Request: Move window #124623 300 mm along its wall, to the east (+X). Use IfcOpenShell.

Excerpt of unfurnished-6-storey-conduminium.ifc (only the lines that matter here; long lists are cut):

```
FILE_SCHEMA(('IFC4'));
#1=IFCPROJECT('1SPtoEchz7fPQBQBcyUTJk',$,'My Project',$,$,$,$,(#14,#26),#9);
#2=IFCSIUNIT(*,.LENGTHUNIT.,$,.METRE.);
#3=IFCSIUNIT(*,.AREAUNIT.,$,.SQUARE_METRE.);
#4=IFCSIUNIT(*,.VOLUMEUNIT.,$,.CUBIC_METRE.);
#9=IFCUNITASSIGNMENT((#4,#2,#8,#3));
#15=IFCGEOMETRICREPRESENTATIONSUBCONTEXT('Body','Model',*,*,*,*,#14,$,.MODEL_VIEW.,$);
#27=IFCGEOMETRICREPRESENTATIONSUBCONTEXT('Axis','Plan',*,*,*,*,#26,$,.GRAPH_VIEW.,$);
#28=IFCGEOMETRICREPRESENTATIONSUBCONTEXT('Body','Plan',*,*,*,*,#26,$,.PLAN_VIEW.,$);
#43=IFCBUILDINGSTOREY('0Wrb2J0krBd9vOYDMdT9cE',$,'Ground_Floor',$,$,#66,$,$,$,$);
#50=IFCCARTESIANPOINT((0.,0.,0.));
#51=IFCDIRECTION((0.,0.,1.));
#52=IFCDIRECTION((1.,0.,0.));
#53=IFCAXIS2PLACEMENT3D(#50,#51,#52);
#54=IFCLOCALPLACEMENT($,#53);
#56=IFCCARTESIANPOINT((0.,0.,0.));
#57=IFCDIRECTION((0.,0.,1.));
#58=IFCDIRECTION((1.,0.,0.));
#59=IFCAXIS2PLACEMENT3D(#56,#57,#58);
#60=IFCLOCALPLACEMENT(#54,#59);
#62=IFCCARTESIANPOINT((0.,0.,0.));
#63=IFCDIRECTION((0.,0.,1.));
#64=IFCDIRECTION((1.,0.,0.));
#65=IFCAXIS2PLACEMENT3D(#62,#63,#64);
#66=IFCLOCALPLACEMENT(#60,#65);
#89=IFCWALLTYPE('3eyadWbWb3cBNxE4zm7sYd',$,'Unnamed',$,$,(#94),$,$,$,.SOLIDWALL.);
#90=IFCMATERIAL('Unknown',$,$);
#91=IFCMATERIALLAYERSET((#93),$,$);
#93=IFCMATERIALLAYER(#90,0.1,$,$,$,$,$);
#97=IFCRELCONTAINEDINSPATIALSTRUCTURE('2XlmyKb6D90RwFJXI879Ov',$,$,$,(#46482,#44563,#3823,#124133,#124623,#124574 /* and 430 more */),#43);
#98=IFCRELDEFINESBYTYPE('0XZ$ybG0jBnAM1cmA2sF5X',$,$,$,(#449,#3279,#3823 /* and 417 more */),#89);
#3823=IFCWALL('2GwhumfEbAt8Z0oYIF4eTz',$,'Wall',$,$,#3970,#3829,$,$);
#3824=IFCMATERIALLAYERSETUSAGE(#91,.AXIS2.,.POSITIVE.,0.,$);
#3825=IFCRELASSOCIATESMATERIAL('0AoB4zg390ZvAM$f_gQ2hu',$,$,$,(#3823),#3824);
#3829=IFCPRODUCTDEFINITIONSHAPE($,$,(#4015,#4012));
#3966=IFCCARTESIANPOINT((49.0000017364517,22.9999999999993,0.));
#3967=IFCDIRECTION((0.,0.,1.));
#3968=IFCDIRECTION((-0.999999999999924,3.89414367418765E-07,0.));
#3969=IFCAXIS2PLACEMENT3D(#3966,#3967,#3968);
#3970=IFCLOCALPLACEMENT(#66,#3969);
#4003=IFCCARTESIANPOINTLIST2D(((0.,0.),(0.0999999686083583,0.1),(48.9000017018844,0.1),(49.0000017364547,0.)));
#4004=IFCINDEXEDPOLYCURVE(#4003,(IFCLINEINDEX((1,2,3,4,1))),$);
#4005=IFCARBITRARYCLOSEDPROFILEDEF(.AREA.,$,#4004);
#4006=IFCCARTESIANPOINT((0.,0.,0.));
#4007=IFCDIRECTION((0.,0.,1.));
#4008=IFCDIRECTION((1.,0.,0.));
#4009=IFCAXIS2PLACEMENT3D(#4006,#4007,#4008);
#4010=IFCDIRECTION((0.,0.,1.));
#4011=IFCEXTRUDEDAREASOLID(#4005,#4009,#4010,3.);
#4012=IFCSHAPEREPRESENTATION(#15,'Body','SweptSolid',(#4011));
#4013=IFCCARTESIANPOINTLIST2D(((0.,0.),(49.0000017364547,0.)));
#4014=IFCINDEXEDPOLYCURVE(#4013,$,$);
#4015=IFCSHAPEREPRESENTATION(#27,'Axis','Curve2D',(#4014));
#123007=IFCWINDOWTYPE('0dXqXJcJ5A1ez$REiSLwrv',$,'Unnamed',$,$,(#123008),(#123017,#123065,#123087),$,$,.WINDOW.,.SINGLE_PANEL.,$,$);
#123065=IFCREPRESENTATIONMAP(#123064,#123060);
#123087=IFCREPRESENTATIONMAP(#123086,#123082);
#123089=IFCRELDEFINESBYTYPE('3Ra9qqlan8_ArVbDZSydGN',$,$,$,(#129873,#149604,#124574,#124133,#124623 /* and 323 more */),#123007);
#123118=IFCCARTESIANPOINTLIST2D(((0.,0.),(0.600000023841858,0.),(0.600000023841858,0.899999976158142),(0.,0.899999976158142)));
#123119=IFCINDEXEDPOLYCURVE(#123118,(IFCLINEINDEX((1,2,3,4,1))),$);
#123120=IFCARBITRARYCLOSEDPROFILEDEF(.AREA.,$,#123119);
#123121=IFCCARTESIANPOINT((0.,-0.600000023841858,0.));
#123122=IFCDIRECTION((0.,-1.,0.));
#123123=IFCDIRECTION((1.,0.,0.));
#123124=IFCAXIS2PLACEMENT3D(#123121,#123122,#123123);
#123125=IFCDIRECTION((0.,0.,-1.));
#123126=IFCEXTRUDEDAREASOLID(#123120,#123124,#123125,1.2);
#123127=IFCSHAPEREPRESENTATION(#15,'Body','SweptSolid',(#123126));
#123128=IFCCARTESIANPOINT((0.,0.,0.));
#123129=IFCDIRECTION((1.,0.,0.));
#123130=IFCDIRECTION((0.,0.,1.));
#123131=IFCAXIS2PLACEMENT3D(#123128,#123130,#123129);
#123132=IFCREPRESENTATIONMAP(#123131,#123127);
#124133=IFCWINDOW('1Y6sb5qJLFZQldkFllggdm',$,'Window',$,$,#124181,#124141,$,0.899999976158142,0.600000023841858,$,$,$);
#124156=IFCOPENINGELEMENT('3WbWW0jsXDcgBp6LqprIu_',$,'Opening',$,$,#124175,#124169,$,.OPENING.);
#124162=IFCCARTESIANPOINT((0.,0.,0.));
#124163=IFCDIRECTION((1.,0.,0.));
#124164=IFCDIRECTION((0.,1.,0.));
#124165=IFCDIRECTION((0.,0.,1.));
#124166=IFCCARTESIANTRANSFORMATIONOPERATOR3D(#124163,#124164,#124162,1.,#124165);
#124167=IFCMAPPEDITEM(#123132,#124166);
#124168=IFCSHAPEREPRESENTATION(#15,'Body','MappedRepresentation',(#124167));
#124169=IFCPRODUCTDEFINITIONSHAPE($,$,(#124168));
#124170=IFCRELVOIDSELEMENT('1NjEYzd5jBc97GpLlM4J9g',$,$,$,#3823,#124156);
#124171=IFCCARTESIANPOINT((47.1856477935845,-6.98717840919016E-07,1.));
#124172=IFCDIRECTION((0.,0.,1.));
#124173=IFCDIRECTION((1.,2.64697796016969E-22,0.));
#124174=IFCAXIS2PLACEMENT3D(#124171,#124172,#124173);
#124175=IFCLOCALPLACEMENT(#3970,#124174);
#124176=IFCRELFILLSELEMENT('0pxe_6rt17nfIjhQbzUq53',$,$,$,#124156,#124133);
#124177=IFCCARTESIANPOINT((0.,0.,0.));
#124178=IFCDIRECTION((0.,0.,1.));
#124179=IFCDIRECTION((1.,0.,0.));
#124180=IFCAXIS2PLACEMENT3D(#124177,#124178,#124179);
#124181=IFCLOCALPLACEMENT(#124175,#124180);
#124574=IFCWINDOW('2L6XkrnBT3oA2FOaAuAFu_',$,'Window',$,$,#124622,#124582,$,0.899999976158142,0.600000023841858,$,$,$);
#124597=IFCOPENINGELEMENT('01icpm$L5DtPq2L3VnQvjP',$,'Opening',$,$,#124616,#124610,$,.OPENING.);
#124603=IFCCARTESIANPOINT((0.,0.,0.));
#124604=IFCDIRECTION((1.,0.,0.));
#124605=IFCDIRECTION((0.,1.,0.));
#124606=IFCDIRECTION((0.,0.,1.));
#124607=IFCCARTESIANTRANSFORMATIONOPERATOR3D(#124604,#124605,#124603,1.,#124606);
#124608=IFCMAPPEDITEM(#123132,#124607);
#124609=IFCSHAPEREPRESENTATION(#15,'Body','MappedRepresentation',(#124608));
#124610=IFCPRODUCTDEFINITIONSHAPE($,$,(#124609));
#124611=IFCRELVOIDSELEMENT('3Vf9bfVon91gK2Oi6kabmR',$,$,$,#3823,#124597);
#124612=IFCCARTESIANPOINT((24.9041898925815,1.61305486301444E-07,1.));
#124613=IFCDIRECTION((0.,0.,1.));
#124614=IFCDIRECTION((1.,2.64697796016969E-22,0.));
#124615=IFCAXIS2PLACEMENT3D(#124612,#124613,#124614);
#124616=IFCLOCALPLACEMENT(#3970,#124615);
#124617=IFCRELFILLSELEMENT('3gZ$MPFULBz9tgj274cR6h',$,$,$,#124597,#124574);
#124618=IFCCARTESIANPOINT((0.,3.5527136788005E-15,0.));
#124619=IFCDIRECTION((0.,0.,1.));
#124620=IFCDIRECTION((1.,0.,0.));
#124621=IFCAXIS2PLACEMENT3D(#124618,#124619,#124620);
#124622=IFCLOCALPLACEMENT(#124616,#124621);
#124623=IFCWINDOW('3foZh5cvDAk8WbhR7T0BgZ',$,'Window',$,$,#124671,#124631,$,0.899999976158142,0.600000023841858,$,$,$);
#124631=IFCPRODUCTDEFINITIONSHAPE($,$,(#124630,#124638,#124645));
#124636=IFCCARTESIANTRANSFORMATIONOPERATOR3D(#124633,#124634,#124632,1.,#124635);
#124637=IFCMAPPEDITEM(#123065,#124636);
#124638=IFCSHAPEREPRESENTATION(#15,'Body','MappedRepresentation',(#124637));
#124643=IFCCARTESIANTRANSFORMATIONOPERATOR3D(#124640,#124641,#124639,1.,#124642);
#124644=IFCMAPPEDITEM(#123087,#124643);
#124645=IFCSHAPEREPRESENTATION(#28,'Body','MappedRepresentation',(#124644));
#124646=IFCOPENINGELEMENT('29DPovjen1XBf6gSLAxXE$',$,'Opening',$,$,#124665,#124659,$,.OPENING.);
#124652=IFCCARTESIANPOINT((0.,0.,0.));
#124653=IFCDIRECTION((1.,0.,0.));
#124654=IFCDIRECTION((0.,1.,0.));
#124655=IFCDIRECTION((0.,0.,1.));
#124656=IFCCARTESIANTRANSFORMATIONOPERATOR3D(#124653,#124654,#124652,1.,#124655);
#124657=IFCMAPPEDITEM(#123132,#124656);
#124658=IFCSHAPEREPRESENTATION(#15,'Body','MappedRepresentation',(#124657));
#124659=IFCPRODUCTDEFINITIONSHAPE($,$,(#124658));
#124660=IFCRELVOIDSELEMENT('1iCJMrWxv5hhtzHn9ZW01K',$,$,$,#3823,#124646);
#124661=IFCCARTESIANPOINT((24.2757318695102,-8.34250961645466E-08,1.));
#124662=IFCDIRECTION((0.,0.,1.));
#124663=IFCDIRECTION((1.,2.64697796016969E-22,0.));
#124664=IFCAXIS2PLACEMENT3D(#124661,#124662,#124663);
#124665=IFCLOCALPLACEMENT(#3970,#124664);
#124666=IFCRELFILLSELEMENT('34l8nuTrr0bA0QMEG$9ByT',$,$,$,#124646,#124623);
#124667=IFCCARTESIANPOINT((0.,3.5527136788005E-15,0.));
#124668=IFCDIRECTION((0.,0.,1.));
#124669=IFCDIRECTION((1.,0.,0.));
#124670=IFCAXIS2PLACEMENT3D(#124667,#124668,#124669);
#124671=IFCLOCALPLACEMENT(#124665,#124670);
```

```python
import ifcopenshell
import ifcopenshell.api.geometry
import ifcopenshell.util.placement

model = ifcopenshell.open("unfurnished-6-storey-conduminium.ifc")

window = model.by_guid("3foZh5cvDAk8WbhR7T0BgZ")
opening = window.FillsVoids[0].RelatingOpeningElement
wall = opening.VoidsElements[0].RelatingBuildingElement

wall_matrix = ifcopenshell.util.placement.get_local_placement(wall.ObjectPlacement)
shift = wall_matrix[:3, 0] * -0.3
before = ifcopenshell.util.placement.get_local_placement(window.ObjectPlacement)[:3, 3].copy()

# The window is placed relative to its opening, so it follows when the opening moves.
matrix = ifcopenshell.util.placement.get_local_placement(opening.ObjectPlacement)
matrix[:3, 3] += shift
ifcopenshell.api.geometry.edit_object_placement(
    model, product=opening, matrix=matrix, is_si=False, should_transform_children=True
)

after = ifcopenshell.util.placement.get_local_placement(window.ObjectPlacement)[:3, 3]
print("window moved by", (after - before).round(3) + 0.0)

model.write("unfurnished-6-storey-conduminium_updated.ifc")
```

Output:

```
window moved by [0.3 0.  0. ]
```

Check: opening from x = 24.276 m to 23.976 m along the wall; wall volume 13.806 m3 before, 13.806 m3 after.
